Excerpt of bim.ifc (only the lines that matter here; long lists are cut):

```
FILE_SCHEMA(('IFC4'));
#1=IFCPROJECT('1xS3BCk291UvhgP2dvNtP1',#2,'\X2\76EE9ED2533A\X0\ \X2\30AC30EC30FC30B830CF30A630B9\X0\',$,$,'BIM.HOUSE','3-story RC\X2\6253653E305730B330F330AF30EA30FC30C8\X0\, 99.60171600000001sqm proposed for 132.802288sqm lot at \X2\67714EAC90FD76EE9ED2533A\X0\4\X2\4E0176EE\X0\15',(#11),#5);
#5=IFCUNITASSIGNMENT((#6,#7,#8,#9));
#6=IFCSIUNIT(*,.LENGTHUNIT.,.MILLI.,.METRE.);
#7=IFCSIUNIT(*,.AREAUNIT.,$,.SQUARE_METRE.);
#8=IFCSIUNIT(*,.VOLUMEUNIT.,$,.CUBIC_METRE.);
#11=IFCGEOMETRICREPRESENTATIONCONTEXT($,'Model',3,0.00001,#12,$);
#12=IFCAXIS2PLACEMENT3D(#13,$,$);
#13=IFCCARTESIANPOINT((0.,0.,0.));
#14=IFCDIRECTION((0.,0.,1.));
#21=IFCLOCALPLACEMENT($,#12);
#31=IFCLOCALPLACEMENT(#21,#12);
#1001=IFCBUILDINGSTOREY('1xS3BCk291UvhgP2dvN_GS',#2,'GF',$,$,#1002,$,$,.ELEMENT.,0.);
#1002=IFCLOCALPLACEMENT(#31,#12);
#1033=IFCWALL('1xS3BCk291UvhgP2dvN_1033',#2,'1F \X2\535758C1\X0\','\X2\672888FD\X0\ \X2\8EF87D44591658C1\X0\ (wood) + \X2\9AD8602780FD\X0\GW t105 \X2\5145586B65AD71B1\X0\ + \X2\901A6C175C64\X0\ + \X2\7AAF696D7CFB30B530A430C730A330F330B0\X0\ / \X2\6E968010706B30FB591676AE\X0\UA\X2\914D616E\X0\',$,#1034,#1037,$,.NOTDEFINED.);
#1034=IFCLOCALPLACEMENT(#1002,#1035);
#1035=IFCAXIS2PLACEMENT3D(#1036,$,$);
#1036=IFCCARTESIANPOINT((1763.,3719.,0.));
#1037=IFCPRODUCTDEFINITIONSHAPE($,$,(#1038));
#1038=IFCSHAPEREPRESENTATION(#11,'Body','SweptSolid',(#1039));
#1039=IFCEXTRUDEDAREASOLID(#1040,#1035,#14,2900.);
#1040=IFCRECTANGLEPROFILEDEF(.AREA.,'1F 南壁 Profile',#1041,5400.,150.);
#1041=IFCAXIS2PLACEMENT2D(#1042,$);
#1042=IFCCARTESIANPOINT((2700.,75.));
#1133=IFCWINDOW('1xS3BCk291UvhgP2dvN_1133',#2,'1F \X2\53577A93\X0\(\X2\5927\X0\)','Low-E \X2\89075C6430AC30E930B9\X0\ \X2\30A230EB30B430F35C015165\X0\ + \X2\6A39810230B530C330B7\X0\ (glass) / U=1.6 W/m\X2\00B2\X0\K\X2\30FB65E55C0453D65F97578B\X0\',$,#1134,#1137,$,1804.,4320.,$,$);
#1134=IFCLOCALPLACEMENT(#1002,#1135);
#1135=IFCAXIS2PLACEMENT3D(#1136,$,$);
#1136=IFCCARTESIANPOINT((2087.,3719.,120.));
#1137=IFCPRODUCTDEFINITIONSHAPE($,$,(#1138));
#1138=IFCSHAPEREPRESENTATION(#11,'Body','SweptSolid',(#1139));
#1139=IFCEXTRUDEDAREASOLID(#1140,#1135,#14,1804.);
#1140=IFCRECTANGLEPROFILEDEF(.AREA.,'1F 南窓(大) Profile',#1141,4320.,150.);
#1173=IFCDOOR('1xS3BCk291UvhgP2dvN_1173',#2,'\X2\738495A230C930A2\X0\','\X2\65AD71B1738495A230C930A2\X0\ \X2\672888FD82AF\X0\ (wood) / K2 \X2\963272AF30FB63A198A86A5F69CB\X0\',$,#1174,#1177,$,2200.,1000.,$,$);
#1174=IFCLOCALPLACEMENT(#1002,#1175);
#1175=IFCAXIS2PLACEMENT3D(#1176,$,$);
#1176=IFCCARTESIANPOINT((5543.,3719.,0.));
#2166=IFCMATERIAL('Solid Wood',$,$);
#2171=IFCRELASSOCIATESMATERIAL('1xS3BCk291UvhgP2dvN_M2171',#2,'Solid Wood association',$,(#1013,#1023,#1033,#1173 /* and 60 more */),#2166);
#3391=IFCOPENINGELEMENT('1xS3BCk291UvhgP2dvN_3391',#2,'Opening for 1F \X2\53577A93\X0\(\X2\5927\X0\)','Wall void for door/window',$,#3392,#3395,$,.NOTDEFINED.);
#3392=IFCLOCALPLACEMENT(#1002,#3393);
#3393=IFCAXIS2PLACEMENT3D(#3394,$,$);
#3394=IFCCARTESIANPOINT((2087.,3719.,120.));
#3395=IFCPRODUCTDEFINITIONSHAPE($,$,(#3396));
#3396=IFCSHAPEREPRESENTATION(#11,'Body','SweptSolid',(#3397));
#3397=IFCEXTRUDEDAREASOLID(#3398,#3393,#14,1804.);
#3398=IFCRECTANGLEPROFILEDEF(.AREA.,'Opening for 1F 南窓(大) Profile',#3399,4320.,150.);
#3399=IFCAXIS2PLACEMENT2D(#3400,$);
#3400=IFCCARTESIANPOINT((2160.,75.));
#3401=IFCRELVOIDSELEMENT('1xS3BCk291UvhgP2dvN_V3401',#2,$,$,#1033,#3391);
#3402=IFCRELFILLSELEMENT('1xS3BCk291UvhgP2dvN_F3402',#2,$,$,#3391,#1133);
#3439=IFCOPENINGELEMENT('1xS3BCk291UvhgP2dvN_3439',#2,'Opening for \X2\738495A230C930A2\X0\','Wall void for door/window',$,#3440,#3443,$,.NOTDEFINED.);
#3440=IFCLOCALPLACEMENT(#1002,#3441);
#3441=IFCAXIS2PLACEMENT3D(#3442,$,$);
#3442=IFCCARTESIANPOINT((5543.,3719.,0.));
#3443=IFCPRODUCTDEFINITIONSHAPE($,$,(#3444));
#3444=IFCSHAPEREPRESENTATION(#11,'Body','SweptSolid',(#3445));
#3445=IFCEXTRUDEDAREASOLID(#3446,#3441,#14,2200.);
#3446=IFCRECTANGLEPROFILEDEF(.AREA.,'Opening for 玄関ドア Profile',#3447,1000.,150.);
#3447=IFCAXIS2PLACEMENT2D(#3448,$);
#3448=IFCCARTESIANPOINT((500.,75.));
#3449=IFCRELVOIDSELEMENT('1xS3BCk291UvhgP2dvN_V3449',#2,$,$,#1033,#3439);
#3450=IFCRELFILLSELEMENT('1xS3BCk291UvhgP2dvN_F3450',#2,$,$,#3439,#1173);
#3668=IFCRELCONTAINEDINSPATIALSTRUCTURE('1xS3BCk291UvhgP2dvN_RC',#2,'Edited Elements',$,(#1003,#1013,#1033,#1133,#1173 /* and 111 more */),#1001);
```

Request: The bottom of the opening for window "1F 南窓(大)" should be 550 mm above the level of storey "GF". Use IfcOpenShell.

```python
import numpy as np
import ifcopenshell
import ifcopenshell.api.geometry
import ifcopenshell.geom
import ifcopenshell.util.element
import ifcopenshell.util.placement
import ifcopenshell.util.shape
import ifcopenshell.util.unit

model = ifcopenshell.open("bim.ifc")
unit_scale = ifcopenshell.util.unit.calculate_unit_scale(model)

window = model.by_id(1133)
opening = window.FillsVoids[0].RelatingOpeningElement
storey = ifcopenshell.util.element.get_container(window, ifc_class="IfcBuildingStorey")
level = ifcopenshell.util.placement.get_local_placement(storey.ObjectPlacement)[2, 3]

# The opening's origin need not be at the sill, so measure its lowest point.
shape = ifcopenshell.geom.create_shape(ifcopenshell.geom.settings(), opening)
bottom = ifcopenshell.util.shape.get_shape_bottom_elevation(shape, shape.geometry) / unit_scale
dz = level + 0.55 / unit_scale - bottom

shift = np.array([0.0, 0.0, dz])
# The window is not placed relative to its opening, so move both.
for product in (opening, window):
    matrix = ifcopenshell.util.placement.get_local_placement(product.ObjectPlacement)
    matrix[:3, 3] += shift
    ifcopenshell.api.geometry.edit_object_placement(model, product=product, matrix=matrix, is_si=False)

print(f"moved by {dz * unit_scale:+.3f} m")

model.write("bim-out.ifc")
```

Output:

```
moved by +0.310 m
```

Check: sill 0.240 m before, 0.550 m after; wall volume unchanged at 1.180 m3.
